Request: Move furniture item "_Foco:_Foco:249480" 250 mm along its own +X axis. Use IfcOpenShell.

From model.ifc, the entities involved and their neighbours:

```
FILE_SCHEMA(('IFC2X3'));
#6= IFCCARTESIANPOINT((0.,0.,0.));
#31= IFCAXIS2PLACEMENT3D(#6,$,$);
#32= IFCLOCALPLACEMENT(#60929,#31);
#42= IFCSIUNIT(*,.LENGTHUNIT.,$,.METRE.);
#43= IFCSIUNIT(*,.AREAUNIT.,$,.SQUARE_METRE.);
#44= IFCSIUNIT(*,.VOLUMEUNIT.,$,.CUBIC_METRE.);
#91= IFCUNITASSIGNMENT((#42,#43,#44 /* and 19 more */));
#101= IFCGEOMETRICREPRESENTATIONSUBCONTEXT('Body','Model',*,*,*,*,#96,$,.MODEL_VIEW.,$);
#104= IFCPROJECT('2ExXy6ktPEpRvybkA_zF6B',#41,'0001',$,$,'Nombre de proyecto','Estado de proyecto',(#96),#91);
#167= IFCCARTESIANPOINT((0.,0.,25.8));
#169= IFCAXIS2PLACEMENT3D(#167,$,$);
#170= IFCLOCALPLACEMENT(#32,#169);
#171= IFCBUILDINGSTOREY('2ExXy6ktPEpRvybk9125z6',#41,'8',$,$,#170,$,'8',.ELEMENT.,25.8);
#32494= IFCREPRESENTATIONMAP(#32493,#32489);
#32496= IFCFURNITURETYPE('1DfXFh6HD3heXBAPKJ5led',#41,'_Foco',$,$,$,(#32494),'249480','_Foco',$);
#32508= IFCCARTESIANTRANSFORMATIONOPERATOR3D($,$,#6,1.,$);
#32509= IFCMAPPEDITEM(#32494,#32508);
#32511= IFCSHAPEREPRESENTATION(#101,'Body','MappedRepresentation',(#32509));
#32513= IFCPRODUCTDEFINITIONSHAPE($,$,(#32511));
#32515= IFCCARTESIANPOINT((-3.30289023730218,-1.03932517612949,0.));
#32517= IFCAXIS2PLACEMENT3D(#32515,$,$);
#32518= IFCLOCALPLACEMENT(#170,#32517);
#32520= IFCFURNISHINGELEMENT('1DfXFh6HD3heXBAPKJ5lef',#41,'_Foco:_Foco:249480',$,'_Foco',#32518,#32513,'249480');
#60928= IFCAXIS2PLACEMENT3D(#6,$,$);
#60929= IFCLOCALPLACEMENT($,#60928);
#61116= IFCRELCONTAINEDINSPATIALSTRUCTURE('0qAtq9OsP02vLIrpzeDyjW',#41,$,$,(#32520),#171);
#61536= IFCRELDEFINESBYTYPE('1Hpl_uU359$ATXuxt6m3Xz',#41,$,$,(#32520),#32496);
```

```python
import ifcopenshell
import ifcopenshell.api.geometry
import ifcopenshell.util.placement
import ifcopenshell.util.unit

model = ifcopenshell.open("model.ifc")
unit_scale = ifcopenshell.util.unit.calculate_unit_scale(model)

item = model.by_guid("1DfXFh6HD3heXBAPKJ5lef")
matrix = ifcopenshell.util.placement.get_local_placement(item.ObjectPlacement)
matrix[:3, 3] += matrix[:3, 0] * 0.25 / unit_scale
ifcopenshell.api.geometry.edit_object_placement(model, product=item, matrix=matrix, is_si=False)

print(ifcopenshell.util.placement.get_local_placement(item.ObjectPlacement).round(3) + 0.0)

model.write("model_rev.ifc")
```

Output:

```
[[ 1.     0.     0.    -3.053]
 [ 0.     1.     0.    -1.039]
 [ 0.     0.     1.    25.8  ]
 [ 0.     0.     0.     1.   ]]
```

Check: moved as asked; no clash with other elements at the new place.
